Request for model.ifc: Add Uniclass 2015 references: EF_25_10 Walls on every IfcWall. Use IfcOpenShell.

First a look at what the model holds.

```python
import ifcopenshell

model = ifcopenshell.open("model.ifc")
print(model.schema)
print("classifications:", [c.Name for c in model.by_type("IfcClassification")])
for ifc_class in ("IfcDoor", "IfcRoof", "IfcStair", "IfcWall", "IfcWindow"):
    print(ifc_class, len(model.by_type(ifc_class)))
```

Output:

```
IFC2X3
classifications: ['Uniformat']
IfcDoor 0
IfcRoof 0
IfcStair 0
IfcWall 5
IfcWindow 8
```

```python
import ifcopenshell
import ifcopenshell.api.classification

model = ifcopenshell.open("model.ifc")

# IFC2X3 requires Source and Edition and has no link from the project to the system.
system = model.create_entity("IfcClassification", Source="NBS", Edition="2015", Name="Uniclass 2015")

codes = {
    "IfcWall": ("EF_25_10", "Walls"),
}
for ifc_class, (code, name) in codes.items():
    products = model.by_type(ifc_class)
    ifcopenshell.api.classification.add_reference(
        model, products=products, classification=system, identification=code, name=name
    )
    print(code, len(products))

model.write("model_updated.ifc")
```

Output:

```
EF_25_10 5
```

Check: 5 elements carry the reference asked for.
